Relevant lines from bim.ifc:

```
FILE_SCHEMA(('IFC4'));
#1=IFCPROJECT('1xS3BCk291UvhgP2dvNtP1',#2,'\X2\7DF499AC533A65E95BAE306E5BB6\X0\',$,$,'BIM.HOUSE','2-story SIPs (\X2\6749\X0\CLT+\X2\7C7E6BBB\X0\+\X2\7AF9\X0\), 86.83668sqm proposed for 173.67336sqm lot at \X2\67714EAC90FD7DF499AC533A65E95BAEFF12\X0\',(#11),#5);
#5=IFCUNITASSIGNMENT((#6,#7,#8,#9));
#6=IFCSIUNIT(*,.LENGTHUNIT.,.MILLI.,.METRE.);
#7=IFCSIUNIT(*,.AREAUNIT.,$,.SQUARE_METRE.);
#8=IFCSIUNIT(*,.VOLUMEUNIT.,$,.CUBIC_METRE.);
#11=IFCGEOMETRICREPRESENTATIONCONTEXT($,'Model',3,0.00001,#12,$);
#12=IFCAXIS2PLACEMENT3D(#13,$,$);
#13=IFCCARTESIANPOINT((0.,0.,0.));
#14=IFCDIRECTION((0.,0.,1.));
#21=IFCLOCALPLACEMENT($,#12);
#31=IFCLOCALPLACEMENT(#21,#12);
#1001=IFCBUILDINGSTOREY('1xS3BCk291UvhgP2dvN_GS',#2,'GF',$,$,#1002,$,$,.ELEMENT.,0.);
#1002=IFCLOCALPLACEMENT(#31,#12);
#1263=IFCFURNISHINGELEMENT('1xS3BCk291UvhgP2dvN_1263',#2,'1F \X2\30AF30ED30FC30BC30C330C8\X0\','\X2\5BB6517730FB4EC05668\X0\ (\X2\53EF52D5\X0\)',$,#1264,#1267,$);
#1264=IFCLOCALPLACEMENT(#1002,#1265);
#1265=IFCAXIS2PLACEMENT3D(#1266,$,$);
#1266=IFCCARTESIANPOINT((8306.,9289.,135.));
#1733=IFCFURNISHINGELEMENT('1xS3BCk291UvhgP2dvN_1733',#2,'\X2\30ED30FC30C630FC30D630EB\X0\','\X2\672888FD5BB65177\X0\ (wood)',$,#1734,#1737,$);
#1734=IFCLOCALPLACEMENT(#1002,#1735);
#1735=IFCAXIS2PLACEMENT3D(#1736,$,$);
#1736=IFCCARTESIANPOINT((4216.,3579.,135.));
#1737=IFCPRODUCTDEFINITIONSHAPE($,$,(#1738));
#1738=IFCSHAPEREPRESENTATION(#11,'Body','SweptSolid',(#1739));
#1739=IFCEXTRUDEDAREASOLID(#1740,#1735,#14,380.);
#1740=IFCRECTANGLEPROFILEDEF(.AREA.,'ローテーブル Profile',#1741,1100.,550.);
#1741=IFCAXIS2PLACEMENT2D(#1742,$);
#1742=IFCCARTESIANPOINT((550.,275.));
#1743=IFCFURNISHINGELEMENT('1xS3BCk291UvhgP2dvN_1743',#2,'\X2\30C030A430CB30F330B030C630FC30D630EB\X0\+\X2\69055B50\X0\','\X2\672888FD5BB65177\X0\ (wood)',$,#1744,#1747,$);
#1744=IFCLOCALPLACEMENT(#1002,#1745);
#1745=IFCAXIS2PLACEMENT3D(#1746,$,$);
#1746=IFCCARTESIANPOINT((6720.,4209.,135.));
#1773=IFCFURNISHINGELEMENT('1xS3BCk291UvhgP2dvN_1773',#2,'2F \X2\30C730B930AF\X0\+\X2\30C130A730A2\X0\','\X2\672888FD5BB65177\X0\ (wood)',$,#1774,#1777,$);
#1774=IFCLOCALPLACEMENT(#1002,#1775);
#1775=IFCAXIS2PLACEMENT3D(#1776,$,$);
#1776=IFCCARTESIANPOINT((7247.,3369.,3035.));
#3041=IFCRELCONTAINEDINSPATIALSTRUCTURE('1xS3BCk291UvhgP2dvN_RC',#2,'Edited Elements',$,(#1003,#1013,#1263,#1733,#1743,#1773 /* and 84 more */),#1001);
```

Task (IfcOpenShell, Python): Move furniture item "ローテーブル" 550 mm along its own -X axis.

```python
import ifcopenshell
import ifcopenshell.api.geometry
import ifcopenshell.util.placement

model = ifcopenshell.open("bim.ifc")

item = model.by_guid("1xS3BCk291UvhgP2dvN_1733")
matrix = ifcopenshell.util.placement.get_local_placement(item.ObjectPlacement)
matrix[:3, 3] -= matrix[:3, 0] * 550.0
ifcopenshell.api.geometry.edit_object_placement(model, product=item, matrix=matrix, is_si=False)

print(ifcopenshell.util.placement.get_local_placement(item.ObjectPlacement).round(3) + 0.0)

model.write("bim_updated.ifc")
```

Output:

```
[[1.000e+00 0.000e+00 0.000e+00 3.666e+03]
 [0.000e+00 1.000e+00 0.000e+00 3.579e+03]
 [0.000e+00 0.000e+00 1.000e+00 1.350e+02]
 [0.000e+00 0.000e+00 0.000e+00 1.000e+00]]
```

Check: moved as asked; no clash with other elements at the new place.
